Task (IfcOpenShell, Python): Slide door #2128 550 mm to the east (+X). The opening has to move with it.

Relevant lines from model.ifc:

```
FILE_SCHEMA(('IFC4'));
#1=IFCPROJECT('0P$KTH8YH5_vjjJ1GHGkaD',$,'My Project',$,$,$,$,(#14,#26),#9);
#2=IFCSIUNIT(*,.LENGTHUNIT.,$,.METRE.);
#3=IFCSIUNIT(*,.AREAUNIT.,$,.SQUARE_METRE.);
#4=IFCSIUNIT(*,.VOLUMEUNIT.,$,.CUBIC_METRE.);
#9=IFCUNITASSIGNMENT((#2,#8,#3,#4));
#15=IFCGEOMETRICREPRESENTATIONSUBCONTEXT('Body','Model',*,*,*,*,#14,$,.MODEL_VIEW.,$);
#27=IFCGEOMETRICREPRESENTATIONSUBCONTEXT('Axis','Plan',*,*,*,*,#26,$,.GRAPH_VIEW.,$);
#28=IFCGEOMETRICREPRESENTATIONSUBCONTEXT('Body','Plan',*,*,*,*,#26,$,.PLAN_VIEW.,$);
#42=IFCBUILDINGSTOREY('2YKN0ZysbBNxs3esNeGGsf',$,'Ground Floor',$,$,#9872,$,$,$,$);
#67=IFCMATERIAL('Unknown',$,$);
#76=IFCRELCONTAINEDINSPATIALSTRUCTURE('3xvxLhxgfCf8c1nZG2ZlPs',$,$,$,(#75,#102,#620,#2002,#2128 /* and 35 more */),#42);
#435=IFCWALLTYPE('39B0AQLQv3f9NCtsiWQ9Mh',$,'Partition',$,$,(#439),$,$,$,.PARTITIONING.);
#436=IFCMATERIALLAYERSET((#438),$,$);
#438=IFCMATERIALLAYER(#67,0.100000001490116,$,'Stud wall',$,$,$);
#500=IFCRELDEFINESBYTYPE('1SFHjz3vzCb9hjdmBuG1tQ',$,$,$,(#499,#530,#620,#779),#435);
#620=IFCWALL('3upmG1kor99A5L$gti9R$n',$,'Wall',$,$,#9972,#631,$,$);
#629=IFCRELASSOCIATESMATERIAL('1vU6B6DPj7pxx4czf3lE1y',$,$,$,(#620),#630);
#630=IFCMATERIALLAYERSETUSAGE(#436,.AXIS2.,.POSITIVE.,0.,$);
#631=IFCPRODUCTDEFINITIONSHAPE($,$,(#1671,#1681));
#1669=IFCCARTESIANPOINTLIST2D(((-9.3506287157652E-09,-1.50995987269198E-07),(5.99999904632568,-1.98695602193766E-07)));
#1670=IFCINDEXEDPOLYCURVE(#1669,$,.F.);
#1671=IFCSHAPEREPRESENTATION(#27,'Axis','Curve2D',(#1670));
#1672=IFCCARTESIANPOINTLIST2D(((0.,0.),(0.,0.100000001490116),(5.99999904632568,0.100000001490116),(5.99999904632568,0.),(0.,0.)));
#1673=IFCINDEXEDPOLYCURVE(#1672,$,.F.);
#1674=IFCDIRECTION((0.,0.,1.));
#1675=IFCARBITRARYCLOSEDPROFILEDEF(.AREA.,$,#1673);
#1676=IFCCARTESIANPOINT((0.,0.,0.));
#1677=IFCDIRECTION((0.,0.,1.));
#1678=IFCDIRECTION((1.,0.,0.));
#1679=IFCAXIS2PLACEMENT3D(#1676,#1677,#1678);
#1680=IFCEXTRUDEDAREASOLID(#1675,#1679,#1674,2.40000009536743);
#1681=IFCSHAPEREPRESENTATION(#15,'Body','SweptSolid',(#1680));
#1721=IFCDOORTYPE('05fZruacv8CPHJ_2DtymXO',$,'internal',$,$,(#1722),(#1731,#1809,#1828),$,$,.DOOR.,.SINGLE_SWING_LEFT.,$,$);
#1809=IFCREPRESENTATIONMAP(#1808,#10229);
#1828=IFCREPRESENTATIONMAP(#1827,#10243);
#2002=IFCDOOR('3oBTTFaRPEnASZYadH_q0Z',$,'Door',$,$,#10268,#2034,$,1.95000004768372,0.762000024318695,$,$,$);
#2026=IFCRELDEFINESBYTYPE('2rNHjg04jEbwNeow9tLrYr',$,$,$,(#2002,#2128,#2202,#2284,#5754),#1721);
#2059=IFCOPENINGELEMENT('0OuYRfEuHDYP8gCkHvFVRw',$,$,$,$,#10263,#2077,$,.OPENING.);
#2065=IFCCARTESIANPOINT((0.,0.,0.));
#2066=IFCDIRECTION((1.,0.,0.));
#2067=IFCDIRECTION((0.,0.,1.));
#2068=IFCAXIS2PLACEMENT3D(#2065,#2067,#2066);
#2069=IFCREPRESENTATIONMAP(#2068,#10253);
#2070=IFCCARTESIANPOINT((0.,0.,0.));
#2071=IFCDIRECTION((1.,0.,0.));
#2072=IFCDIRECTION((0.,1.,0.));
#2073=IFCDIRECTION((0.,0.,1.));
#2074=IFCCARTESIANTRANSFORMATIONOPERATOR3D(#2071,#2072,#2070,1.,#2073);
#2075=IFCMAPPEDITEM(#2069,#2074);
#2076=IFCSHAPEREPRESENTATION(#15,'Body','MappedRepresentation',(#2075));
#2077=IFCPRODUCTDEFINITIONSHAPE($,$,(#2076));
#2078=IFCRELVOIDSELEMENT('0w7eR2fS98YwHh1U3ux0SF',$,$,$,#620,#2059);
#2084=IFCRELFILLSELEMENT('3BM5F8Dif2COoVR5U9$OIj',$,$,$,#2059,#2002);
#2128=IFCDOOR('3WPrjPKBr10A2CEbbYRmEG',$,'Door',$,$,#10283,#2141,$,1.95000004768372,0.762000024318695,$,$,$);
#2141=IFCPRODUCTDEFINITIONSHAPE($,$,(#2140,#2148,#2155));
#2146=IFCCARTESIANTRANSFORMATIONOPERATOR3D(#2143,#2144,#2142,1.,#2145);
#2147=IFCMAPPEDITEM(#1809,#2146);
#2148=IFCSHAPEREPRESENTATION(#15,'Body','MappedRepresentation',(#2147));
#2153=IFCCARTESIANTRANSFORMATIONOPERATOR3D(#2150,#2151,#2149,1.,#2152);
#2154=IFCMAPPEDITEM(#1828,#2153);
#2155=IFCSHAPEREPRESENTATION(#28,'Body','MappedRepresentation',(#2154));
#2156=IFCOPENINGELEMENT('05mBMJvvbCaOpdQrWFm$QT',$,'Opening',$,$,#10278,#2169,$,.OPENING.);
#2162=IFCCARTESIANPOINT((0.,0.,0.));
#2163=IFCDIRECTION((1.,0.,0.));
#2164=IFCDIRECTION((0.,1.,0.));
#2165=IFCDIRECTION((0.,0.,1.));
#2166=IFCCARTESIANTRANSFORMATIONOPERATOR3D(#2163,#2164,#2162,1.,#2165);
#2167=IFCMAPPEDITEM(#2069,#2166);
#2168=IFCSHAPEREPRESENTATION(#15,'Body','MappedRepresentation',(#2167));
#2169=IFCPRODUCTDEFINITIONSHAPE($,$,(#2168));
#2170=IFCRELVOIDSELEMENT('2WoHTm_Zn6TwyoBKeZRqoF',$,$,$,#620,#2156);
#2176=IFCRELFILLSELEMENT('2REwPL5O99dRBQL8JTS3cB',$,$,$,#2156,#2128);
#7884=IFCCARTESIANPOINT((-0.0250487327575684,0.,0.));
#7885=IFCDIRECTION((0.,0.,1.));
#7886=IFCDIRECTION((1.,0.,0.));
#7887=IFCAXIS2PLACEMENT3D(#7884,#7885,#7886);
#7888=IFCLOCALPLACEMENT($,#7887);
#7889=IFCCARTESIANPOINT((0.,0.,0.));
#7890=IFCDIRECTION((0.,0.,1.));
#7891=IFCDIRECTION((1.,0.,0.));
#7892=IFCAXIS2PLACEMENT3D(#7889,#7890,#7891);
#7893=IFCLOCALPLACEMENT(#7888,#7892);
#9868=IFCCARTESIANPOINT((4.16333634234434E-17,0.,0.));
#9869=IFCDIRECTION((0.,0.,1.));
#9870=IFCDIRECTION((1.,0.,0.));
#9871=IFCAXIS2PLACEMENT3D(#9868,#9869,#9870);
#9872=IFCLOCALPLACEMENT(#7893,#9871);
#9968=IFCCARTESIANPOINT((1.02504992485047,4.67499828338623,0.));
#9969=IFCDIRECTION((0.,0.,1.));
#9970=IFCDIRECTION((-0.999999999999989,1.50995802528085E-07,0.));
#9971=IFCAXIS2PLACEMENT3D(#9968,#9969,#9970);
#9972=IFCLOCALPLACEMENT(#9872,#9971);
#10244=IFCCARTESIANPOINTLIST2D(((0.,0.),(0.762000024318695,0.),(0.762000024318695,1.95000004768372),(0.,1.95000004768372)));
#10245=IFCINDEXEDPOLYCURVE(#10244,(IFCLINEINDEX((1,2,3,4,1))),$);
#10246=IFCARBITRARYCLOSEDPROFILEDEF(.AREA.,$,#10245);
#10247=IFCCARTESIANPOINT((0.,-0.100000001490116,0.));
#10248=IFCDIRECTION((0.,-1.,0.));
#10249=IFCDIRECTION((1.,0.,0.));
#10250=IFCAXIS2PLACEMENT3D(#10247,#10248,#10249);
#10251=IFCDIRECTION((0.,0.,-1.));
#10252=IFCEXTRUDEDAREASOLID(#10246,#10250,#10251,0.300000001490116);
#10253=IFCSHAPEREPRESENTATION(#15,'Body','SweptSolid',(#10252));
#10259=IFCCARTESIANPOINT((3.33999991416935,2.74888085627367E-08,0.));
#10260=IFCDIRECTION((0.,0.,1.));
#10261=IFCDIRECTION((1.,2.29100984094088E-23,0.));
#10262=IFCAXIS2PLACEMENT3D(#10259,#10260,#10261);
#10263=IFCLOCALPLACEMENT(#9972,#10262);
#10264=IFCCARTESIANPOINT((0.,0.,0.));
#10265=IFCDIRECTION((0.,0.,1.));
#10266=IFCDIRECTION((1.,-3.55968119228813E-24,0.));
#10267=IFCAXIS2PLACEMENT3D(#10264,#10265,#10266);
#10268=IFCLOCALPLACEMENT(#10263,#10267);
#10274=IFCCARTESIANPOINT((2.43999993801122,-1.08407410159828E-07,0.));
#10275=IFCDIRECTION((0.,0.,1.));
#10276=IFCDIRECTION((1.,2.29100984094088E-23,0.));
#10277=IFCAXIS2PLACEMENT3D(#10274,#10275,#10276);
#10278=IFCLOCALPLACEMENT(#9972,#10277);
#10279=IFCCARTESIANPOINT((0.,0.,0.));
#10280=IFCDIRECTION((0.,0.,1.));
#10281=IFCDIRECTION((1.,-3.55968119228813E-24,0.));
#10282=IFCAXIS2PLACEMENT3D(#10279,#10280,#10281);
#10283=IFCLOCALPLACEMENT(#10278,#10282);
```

```python
import ifcopenshell
import ifcopenshell.api.geometry
import ifcopenshell.util.placement
import ifcopenshell.util.unit

model = ifcopenshell.open("model.ifc")
unit_scale = ifcopenshell.util.unit.calculate_unit_scale(model)

door = model.by_guid("3WPrjPKBr10A2CEbbYRmEG")
opening = door.FillsVoids[0].RelatingOpeningElement
wall = opening.VoidsElements[0].RelatingBuildingElement

wall_matrix = ifcopenshell.util.placement.get_local_placement(wall.ObjectPlacement)
shift = wall_matrix[:3, 0] * -0.55 / unit_scale
before = ifcopenshell.util.placement.get_local_placement(door.ObjectPlacement)[:3, 3].copy()

# The door is placed relative to its opening, so it follows when the opening moves.
matrix = ifcopenshell.util.placement.get_local_placement(opening.ObjectPlacement)
matrix[:3, 3] += shift
ifcopenshell.api.geometry.edit_object_placement(
    model, product=opening, matrix=matrix, is_si=False, should_transform_children=True
)

after = ifcopenshell.util.placement.get_local_placement(door.ObjectPlacement)[:3, 3]
print("door moved by", (after - before).round(3) + 0.0)

model.write("model_v2.ifc")
```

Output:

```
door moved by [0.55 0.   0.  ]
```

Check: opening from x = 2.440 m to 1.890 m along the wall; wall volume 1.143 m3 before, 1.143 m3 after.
